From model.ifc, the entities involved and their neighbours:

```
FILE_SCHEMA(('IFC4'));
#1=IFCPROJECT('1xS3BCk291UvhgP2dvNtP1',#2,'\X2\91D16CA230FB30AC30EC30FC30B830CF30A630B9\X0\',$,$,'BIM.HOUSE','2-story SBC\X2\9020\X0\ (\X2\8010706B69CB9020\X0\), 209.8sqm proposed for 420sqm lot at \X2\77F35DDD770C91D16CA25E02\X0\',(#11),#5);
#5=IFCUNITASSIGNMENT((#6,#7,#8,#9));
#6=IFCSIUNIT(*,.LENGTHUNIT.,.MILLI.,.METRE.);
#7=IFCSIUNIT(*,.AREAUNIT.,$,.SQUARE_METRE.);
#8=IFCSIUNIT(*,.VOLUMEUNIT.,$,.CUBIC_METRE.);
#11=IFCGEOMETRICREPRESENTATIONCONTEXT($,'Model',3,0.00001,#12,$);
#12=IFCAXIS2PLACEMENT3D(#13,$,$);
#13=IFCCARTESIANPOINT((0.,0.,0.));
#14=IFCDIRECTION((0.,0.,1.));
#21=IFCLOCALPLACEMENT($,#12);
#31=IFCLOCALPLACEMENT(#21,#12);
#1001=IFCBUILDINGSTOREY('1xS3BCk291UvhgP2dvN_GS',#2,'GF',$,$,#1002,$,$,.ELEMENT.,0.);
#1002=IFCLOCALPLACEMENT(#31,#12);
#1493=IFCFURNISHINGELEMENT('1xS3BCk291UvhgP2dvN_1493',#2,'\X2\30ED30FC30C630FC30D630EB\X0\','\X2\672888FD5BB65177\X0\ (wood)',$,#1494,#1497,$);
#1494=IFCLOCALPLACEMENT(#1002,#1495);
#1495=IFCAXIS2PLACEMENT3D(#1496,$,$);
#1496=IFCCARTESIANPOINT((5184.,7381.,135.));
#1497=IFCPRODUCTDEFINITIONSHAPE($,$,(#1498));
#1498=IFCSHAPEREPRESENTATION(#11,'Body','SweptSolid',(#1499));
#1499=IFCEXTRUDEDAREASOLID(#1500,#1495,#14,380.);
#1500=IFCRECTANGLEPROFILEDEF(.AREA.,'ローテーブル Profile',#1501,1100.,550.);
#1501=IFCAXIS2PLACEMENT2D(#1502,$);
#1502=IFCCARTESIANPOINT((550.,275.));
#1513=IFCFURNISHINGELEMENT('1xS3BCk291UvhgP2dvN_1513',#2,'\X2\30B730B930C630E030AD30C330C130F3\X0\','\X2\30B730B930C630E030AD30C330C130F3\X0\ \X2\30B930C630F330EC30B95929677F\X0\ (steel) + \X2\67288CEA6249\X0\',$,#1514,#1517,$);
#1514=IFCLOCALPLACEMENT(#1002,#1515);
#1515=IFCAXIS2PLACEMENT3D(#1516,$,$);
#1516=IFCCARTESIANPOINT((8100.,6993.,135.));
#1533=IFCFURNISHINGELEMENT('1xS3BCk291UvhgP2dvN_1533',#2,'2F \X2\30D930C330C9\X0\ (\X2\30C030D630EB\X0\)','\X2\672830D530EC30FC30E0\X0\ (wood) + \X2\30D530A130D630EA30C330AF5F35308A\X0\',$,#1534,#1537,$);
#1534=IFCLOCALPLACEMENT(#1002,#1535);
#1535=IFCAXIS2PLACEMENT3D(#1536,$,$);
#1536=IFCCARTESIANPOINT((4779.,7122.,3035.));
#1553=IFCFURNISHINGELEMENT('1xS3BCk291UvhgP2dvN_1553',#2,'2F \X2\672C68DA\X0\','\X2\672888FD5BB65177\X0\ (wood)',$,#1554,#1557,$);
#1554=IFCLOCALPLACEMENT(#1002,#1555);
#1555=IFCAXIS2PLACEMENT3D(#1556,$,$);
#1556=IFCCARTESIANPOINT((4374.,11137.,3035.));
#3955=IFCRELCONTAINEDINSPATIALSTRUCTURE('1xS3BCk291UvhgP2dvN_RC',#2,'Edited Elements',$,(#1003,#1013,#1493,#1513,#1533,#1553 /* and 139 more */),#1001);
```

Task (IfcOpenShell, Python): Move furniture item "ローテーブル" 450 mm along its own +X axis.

```python
import ifcopenshell
import ifcopenshell.api.geometry
import ifcopenshell.util.placement

model = ifcopenshell.open("model.ifc")

item = model.by_guid("1xS3BCk291UvhgP2dvN_1493")
matrix = ifcopenshell.util.placement.get_local_placement(item.ObjectPlacement)
matrix[:3, 3] += matrix[:3, 0] * 450.0
ifcopenshell.api.geometry.edit_object_placement(model, product=item, matrix=matrix, is_si=False)

print(ifcopenshell.util.placement.get_local_placement(item.ObjectPlacement).round(3) + 0.0)

model.write("model_v2.ifc")
```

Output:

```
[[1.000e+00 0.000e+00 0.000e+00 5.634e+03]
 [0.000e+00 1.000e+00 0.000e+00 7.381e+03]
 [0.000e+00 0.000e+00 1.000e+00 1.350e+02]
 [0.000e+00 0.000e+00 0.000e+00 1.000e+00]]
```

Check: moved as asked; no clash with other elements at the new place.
